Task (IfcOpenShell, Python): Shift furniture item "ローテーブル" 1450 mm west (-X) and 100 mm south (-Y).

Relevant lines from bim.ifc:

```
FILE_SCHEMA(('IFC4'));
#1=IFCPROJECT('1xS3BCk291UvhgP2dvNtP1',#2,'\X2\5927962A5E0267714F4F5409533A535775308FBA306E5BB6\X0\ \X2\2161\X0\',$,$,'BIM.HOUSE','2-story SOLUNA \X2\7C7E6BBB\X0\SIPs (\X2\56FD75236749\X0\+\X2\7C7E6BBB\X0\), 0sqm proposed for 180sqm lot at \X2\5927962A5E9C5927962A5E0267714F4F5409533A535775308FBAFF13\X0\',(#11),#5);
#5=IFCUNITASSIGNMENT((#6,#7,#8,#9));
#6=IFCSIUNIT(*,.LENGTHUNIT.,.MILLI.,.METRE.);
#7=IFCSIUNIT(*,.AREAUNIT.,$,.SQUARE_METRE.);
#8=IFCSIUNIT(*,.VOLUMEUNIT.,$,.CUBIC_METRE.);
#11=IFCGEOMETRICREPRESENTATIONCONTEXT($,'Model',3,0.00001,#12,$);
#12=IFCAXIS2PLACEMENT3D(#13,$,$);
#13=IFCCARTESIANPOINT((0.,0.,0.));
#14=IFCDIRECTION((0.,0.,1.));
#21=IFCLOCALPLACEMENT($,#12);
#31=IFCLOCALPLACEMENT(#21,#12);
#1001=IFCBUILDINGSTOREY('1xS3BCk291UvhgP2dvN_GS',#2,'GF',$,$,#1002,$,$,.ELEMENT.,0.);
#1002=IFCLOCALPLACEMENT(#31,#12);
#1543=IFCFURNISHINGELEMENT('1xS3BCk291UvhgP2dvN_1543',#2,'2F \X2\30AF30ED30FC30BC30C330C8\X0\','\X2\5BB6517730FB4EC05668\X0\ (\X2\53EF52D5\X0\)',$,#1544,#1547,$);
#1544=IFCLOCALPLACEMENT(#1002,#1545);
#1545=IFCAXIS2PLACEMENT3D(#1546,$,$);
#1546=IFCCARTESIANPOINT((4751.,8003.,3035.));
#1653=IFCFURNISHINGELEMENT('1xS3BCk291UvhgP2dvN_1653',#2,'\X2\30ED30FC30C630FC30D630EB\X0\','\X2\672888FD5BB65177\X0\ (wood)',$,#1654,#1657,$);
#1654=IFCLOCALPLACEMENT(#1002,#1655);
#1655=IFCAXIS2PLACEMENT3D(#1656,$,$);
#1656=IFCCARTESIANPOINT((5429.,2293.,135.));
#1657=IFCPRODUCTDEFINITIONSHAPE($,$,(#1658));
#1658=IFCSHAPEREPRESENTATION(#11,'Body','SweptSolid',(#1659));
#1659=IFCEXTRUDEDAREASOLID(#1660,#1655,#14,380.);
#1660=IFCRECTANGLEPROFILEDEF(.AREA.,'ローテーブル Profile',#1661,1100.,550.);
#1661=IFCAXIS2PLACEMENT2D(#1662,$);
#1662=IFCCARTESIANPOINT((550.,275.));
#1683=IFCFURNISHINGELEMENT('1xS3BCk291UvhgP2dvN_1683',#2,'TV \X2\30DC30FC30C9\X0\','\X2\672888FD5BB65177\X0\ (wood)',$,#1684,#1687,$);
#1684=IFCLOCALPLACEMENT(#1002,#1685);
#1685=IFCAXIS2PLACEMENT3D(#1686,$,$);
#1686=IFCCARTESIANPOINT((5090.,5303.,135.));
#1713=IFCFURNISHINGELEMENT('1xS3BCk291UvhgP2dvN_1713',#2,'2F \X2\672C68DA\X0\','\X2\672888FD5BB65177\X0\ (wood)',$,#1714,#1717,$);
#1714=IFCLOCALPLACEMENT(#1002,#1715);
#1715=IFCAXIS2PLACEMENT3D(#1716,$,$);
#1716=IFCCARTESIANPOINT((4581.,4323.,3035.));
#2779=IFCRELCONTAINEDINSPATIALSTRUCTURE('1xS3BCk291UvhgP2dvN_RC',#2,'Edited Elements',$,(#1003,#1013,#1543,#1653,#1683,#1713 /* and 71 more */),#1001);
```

```python
import ifcopenshell
import ifcopenshell.api.geometry
import ifcopenshell.util.placement
import ifcopenshell.util.unit

model = ifcopenshell.open("bim.ifc")
unit_scale = ifcopenshell.util.unit.calculate_unit_scale(model)

item = model.by_id(1653)
matrix = ifcopenshell.util.placement.get_local_placement(item.ObjectPlacement)
matrix[0, 3] -= 1.45 / unit_scale
matrix[1, 3] -= 0.1 / unit_scale
ifcopenshell.api.geometry.edit_object_placement(model, product=item, matrix=matrix, is_si=False)

print(ifcopenshell.util.placement.get_local_placement(item.ObjectPlacement).round(3) + 0.0)

model.write("bim_edited.ifc")
```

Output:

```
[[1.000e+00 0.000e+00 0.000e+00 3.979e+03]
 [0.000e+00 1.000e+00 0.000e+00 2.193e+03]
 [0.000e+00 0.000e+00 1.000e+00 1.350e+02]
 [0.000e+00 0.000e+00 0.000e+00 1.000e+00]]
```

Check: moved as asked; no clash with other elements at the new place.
